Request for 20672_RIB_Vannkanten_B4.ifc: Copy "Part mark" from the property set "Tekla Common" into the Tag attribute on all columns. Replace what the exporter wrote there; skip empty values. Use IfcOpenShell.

First a look at what the model holds.

```python
import ifcopenshell
import ifcopenshell.util.element

model = ifcopenshell.open("20672_RIB_Vannkanten_B4.ifc")
print(model.schema)
columns = model.by_type("IfcColumn")
print(len(columns), "columns")
for e in columns[:8]:
    source = ifcopenshell.util.element.get_pset(e, "Tekla Common", "Part mark")
    target = e.Tag
    print(e.id(), repr(source), repr(target), sep=" | ")
```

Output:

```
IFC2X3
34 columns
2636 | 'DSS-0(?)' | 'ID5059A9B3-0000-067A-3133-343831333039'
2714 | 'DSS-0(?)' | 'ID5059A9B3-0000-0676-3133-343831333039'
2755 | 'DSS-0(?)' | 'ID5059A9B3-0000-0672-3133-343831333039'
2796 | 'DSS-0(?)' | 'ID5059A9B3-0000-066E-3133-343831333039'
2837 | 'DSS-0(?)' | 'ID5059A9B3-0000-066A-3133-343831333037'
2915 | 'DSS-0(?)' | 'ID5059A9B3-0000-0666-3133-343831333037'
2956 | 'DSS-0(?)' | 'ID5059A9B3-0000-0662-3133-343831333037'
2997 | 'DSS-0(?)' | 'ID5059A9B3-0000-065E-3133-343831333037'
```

```python
import ifcopenshell
import ifcopenshell.util.element

model = ifcopenshell.open("20672_RIB_Vannkanten_B4.ifc")

count = 0
for e in model.by_type("IfcColumn"):
    value = ifcopenshell.util.element.get_pset(e, "Tekla Common", "Part mark")
    current = e.Tag
    if not value or not value.strip() or current == value:
        continue
    e.Tag = value
    count += 1

print(count, "columns updated")

model.write("20672_RIB_Vannkanten_B4_v2.ifc")
```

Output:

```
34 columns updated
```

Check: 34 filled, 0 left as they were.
